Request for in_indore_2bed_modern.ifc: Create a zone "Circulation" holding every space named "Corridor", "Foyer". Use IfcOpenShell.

First a look at what the model holds.

```python
import ifcopenshell

model = ifcopenshell.open("in_indore_2bed_modern.ifc")
print(model.schema)
seen = {}
for space in model.by_type("IfcSpace"):
    seen[space.LongName] = seen.get(space.LongName, 0) + 1
for name, count in sorted(seen.items(), key=str):
    print(count, "x", name)
print("zones:", [z.Name for z in model.by_type("IfcZone")][:20])
```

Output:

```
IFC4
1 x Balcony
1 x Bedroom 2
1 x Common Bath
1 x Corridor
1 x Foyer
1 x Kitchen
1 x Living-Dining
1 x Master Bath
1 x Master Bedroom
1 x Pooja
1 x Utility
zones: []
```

```python
import ifcopenshell
import ifcopenshell.api.group
import ifcopenshell.api.root

model = ifcopenshell.open("in_indore_2bed_modern.ifc")

names = {"Corridor", "Foyer"}
spaces = [s for s in model.by_type("IfcSpace") if s.LongName in names]

zone = ifcopenshell.api.root.create_entity(model, ifc_class="IfcZone", name="Circulation")
ifcopenshell.api.group.assign_group(model, products=spaces, group=zone)
print(len(spaces), "spaces in", zone.Name)

model.write("in_indore_2bed_modern_updated.ifc")
```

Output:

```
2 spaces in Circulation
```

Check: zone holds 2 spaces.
